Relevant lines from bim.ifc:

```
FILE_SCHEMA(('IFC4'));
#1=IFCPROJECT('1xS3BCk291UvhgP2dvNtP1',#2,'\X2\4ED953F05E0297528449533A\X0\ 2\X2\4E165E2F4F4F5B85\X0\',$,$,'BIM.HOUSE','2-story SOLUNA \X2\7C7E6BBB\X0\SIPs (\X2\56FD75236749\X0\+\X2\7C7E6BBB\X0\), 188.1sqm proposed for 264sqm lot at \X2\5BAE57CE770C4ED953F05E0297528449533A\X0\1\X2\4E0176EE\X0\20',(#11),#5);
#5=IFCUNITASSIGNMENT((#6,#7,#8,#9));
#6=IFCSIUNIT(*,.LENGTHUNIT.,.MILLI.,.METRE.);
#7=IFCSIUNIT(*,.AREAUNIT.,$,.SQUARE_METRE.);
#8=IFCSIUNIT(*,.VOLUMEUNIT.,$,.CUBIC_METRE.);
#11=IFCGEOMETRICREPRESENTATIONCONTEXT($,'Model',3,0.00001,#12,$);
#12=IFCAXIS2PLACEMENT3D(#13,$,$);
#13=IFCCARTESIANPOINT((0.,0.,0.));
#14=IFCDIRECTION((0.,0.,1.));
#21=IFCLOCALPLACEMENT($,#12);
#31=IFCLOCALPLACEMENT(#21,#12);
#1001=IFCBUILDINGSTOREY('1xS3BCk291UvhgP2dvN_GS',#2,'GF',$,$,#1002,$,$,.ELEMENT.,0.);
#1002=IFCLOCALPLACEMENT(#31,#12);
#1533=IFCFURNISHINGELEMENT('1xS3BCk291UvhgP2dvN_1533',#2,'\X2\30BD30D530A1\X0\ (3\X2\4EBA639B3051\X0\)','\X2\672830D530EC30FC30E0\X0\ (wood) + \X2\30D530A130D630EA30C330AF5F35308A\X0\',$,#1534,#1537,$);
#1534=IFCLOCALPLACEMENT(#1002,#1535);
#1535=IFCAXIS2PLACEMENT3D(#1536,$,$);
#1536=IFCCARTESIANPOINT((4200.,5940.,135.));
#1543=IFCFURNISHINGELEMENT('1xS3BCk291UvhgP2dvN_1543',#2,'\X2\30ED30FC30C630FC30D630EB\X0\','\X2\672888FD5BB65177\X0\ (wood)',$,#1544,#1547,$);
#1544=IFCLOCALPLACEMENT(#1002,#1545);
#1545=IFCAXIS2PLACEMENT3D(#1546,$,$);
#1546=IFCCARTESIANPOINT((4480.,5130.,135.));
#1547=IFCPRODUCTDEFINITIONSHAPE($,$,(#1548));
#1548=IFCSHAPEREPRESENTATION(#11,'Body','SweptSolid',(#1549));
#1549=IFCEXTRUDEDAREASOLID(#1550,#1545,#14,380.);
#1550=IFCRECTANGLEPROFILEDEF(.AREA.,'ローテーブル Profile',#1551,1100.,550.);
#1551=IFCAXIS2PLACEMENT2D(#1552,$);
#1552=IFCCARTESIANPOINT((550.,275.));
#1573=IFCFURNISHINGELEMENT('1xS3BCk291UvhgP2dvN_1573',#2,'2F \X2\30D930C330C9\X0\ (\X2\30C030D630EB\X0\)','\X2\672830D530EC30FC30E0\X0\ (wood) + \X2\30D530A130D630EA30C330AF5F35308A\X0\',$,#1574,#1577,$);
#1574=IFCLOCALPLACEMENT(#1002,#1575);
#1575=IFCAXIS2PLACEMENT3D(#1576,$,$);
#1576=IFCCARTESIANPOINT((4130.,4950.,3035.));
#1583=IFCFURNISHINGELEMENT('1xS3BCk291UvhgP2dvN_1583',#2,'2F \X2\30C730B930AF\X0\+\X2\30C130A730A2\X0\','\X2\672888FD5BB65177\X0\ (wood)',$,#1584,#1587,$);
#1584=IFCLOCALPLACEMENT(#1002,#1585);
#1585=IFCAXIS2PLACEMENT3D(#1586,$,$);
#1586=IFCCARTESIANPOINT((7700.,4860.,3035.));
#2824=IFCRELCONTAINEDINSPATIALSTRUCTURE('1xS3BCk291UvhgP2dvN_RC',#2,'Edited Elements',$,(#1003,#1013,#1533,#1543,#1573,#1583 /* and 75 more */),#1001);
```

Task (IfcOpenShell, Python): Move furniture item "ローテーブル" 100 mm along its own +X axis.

```python
import ifcopenshell
import ifcopenshell.api.geometry
import ifcopenshell.util.placement
import ifcopenshell.util.unit

model = ifcopenshell.open("bim.ifc")
unit_scale = ifcopenshell.util.unit.calculate_unit_scale(model)

item = model.by_guid("1xS3BCk291UvhgP2dvN_1543")
matrix = ifcopenshell.util.placement.get_local_placement(item.ObjectPlacement)
matrix[:3, 3] += matrix[:3, 0] * 0.1 / unit_scale
ifcopenshell.api.geometry.edit_object_placement(model, product=item, matrix=matrix, is_si=False)

print(ifcopenshell.util.placement.get_local_placement(item.ObjectPlacement).round(3) + 0.0)

model.write("bim_updated.ifc")
```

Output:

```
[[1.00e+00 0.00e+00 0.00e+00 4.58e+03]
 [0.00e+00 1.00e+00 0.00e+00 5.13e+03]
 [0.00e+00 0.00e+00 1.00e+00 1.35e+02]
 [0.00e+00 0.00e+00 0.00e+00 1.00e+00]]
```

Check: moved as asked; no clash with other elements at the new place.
